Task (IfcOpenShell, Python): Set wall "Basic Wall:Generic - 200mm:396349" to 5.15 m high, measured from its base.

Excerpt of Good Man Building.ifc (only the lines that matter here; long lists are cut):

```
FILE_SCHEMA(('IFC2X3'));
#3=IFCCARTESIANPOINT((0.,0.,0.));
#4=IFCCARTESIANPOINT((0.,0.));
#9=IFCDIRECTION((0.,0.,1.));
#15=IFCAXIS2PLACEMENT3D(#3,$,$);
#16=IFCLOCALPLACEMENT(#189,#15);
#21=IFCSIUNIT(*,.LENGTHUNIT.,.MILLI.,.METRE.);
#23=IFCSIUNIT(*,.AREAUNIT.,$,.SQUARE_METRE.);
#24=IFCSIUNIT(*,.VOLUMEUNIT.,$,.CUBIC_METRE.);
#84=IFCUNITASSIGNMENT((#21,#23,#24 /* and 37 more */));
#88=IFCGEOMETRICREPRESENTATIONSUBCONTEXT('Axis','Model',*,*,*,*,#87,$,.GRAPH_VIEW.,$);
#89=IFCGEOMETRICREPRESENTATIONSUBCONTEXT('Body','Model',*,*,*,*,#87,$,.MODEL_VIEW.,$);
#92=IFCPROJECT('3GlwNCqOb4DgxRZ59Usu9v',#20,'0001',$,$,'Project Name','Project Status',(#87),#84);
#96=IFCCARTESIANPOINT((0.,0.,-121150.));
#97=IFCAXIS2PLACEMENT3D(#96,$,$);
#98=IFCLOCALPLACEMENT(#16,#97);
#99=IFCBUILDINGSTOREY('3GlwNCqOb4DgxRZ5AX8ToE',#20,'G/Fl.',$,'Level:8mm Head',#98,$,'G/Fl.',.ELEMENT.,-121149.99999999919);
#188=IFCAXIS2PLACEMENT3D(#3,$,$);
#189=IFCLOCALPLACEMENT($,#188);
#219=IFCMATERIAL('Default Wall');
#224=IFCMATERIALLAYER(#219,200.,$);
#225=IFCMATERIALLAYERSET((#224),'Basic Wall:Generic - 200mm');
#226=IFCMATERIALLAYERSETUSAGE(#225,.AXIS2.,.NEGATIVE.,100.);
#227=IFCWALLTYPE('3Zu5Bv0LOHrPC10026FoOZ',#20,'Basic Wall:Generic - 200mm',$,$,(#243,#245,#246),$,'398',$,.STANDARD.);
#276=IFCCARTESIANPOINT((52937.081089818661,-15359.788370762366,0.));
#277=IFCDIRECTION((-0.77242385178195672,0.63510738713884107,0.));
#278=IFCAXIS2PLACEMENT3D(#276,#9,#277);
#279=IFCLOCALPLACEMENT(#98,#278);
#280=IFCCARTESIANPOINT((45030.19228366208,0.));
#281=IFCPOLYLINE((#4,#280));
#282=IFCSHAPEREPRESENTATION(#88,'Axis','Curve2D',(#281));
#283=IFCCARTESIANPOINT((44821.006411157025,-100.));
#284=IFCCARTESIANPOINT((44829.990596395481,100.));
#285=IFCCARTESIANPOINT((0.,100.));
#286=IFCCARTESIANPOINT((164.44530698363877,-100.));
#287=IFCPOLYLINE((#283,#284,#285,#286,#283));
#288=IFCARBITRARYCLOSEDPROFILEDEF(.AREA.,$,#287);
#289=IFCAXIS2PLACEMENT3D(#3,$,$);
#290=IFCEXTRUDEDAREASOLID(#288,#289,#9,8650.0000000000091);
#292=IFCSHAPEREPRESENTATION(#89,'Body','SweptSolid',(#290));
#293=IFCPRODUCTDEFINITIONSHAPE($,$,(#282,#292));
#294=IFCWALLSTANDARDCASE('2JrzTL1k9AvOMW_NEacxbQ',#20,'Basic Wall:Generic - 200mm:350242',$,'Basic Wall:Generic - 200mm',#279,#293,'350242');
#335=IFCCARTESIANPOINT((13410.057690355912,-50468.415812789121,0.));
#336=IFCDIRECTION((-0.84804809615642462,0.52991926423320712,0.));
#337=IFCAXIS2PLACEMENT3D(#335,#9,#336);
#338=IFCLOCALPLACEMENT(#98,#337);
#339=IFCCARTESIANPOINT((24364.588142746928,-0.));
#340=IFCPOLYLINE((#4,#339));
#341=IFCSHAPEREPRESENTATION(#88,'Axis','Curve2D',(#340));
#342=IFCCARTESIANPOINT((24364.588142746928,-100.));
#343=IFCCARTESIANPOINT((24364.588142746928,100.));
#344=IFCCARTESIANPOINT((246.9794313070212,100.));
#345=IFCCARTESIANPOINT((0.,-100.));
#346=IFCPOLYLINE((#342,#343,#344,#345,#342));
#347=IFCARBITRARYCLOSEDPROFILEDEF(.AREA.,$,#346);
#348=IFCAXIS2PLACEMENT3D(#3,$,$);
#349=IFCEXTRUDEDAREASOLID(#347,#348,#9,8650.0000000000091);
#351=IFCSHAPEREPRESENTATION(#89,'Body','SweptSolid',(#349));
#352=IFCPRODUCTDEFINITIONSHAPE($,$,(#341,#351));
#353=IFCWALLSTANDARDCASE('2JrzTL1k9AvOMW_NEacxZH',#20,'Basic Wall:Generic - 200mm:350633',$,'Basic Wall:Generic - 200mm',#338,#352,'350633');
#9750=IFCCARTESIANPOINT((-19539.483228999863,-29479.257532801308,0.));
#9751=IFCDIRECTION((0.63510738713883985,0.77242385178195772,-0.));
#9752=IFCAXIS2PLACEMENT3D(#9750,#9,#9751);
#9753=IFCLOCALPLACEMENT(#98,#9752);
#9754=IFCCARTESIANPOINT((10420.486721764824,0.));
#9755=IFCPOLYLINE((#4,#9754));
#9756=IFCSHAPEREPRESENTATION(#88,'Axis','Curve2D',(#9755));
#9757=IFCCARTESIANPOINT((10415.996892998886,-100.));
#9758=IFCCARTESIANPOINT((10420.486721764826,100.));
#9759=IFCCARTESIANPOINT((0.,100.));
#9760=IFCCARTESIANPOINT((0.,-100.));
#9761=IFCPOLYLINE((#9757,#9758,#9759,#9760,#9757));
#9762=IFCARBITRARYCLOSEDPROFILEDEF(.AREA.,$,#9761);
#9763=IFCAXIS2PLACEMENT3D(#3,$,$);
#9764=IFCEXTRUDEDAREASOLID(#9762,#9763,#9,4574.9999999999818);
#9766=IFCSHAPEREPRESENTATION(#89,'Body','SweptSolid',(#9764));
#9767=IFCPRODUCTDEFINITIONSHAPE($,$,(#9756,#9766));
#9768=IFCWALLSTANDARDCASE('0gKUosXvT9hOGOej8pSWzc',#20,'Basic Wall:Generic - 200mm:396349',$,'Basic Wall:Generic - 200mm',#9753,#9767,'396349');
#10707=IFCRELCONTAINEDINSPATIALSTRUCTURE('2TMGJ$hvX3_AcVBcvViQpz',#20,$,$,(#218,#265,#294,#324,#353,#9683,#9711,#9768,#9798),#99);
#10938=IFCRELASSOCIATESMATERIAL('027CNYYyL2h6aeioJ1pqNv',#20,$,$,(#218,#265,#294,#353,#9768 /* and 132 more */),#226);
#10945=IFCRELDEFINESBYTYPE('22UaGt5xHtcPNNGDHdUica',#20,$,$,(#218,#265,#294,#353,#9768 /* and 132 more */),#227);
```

```python
import ifcopenshell
import ifcopenshell.geom
import ifcopenshell.util.representation
import ifcopenshell.util.shape
import ifcopenshell.util.unit

model = ifcopenshell.open("Good Man Building.ifc")
unit_scale = ifcopenshell.util.unit.calculate_unit_scale(model)
settings = ifcopenshell.geom.settings()


def volume(element):
    """Net volume in cubic metres, openings subtracted."""
    shape = ifcopenshell.geom.create_shape(settings, element)
    return ifcopenshell.util.shape.get_volume(shape.geometry)


wall = model.by_guid("0gKUosXvT9hOGOej8pSWzc")
before = volume(wall)

body = ifcopenshell.util.representation.get_representation(wall, "Model", "Body")
solid = body.Items[0]
old_height = solid.Depth
solid.Depth = 5.15 / unit_scale
after = volume(wall)

print(f"height {old_height:g} -> {solid.Depth:g}, volume {before:.3f} -> {after:.3f} m3")

model.write("Good Man Building_rev.ifc")
```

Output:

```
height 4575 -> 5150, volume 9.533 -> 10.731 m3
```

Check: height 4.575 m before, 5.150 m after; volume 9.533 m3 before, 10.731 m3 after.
